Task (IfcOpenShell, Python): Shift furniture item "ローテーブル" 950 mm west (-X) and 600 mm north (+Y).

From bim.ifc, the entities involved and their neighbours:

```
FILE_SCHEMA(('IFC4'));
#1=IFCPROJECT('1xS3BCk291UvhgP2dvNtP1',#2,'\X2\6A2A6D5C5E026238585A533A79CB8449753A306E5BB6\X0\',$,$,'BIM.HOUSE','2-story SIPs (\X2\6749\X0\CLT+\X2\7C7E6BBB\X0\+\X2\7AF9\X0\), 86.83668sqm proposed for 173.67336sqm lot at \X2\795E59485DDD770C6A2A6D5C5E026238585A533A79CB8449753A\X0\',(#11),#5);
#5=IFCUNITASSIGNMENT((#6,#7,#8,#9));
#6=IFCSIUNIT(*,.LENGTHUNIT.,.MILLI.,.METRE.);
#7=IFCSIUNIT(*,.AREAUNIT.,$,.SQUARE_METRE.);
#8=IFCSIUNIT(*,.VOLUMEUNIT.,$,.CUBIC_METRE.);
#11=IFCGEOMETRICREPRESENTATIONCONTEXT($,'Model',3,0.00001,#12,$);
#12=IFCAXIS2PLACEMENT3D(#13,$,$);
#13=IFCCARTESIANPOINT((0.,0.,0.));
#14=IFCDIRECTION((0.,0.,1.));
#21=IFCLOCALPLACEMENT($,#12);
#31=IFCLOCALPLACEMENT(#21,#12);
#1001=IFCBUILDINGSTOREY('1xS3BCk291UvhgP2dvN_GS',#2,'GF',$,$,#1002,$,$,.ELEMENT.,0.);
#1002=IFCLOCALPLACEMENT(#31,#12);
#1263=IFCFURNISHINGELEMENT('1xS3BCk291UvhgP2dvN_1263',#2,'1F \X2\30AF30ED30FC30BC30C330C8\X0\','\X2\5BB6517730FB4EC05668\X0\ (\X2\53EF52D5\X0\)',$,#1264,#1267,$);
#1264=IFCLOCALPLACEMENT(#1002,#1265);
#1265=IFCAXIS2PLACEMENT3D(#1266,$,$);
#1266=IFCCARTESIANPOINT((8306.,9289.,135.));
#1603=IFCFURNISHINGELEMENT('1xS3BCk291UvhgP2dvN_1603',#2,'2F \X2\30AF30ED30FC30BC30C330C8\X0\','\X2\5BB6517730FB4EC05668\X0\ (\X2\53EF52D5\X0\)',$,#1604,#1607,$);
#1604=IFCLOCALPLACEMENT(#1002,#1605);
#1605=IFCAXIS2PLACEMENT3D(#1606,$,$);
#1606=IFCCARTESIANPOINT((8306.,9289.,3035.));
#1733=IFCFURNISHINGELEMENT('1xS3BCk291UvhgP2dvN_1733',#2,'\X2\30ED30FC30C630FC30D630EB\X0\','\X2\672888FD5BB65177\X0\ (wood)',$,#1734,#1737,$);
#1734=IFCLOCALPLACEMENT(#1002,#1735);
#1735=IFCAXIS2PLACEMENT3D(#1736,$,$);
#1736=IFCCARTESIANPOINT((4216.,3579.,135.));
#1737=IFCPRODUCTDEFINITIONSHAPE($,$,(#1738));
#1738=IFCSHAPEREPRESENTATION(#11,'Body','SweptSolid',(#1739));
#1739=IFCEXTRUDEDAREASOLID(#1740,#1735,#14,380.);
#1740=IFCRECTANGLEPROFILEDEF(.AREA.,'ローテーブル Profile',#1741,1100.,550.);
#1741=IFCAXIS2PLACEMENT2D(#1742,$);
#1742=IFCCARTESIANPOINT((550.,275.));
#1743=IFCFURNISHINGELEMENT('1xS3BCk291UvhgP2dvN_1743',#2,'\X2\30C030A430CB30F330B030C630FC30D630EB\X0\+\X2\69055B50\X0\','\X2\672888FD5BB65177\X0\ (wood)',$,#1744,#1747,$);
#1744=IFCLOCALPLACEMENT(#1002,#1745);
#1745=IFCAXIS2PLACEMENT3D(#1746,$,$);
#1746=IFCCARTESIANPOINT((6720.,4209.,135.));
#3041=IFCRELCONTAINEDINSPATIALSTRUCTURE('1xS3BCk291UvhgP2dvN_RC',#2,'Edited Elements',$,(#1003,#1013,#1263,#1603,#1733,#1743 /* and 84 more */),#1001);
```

```python
import ifcopenshell
import ifcopenshell.api.geometry
import ifcopenshell.util.placement

model = ifcopenshell.open("bim.ifc")

item = model.by_guid("1xS3BCk291UvhgP2dvN_1733")
matrix = ifcopenshell.util.placement.get_local_placement(item.ObjectPlacement)
matrix[0, 3] -= 950.0
matrix[1, 3] += 600.0
ifcopenshell.api.geometry.edit_object_placement(model, product=item, matrix=matrix, is_si=False)

print(ifcopenshell.util.placement.get_local_placement(item.ObjectPlacement).round(3) + 0.0)

model.write("bim-out.ifc")
```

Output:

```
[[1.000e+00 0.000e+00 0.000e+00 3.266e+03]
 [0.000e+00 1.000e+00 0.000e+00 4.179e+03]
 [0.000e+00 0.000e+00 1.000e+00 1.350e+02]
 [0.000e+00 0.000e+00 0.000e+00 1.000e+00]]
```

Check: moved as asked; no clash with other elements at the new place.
